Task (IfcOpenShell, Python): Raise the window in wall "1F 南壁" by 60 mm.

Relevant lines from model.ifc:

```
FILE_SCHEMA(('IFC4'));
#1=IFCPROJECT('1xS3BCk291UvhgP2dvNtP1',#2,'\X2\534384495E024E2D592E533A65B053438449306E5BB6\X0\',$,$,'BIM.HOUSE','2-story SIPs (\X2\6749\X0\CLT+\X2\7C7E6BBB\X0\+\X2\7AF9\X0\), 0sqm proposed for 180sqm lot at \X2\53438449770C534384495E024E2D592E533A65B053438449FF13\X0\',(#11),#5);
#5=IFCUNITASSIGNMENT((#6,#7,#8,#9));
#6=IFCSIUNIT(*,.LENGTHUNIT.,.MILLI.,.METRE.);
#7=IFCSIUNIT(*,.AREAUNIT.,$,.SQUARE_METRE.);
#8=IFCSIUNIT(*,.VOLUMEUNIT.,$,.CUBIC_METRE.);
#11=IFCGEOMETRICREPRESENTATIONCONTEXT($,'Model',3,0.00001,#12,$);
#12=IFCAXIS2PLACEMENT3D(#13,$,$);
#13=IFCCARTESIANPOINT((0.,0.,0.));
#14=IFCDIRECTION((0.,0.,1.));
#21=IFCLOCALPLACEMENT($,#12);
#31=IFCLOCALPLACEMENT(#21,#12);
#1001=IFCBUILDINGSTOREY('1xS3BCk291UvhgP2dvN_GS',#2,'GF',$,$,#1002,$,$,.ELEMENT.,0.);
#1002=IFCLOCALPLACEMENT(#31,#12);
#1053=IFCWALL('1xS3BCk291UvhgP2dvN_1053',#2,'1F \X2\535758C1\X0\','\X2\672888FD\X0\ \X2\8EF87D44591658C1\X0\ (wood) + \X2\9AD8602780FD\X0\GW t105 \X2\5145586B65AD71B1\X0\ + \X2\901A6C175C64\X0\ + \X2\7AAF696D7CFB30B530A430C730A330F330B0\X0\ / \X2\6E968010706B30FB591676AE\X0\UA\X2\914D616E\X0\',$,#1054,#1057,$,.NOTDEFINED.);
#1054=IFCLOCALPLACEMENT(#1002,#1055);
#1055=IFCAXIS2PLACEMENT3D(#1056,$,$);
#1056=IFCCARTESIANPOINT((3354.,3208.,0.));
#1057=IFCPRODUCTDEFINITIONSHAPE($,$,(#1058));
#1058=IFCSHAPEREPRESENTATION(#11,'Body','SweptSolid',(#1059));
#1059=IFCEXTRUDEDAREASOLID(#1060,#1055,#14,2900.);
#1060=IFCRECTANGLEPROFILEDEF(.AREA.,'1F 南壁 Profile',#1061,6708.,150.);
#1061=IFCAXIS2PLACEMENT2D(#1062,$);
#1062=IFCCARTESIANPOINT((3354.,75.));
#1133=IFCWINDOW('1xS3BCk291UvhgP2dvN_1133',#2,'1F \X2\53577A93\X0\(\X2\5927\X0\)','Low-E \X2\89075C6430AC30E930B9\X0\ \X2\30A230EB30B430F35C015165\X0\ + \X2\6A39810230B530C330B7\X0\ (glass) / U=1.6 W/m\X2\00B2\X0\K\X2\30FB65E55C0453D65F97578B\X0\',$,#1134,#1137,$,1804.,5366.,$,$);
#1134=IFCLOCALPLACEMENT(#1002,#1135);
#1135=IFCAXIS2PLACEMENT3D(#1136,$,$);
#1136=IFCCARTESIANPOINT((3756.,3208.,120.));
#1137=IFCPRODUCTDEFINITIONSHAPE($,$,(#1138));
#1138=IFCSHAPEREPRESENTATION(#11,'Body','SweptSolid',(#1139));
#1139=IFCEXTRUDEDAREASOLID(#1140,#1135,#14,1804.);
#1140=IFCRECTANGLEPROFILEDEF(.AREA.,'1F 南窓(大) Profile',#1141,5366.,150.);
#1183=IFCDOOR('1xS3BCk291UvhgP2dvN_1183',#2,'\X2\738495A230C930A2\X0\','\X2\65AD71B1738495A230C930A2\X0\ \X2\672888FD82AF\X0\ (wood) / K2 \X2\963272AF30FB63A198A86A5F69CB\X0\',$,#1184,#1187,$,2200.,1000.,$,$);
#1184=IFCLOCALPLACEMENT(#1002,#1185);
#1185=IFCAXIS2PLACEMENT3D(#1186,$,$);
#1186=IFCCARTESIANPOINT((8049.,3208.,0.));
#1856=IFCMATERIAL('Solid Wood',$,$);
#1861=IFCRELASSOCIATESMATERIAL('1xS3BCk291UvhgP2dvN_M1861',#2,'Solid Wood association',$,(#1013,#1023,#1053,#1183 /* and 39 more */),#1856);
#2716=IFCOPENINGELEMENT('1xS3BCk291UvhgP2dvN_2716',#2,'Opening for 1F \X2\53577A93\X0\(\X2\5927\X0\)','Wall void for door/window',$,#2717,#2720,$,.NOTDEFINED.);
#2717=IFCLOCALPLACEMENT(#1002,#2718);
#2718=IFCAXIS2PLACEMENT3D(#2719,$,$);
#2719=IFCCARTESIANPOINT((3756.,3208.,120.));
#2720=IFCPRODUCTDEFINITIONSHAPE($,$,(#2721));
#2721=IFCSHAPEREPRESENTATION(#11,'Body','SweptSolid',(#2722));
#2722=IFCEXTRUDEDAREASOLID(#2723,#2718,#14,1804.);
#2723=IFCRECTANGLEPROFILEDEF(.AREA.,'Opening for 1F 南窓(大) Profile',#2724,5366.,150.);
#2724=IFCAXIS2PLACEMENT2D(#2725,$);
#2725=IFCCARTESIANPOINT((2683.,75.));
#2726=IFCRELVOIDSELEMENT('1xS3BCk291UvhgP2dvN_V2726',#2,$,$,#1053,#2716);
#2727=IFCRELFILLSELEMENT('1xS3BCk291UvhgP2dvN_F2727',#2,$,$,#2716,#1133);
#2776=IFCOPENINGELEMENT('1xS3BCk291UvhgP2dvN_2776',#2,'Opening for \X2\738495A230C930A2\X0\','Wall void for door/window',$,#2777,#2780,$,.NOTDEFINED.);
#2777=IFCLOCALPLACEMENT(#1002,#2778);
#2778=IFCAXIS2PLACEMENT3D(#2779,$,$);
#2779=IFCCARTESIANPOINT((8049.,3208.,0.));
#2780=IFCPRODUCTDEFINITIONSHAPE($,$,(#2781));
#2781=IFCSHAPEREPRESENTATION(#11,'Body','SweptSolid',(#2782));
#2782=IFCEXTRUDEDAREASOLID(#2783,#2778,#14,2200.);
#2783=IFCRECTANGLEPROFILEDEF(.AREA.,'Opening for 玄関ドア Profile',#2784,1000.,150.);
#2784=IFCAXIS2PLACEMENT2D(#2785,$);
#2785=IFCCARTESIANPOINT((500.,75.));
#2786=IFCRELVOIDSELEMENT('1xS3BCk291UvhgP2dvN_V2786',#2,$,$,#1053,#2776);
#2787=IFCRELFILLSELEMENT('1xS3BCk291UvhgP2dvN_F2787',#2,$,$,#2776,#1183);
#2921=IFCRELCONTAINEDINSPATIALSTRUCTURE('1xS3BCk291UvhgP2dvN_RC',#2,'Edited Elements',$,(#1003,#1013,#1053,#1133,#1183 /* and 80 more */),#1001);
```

```python
import numpy as np
import ifcopenshell
import ifcopenshell.api.geometry
import ifcopenshell.util.placement
import ifcopenshell.util.unit

model = ifcopenshell.open("model.ifc")
unit_scale = ifcopenshell.util.unit.calculate_unit_scale(model)

window = model.by_guid("1xS3BCk291UvhgP2dvN_1133")
opening = window.FillsVoids[0].RelatingOpeningElement
dz = 0.06 / unit_scale

shift = np.array([0.0, 0.0, dz])
# The window is not placed relative to its opening, so move both.
for product in (opening, window):
    matrix = ifcopenshell.util.placement.get_local_placement(product.ObjectPlacement)
    matrix[:3, 3] += shift
    ifcopenshell.api.geometry.edit_object_placement(model, product=product, matrix=matrix, is_si=False)

print(f"moved by {dz * unit_scale:+.3f} m")

model.write("model_v2.ifc")
```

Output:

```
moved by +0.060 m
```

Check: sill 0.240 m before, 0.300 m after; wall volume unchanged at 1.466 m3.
